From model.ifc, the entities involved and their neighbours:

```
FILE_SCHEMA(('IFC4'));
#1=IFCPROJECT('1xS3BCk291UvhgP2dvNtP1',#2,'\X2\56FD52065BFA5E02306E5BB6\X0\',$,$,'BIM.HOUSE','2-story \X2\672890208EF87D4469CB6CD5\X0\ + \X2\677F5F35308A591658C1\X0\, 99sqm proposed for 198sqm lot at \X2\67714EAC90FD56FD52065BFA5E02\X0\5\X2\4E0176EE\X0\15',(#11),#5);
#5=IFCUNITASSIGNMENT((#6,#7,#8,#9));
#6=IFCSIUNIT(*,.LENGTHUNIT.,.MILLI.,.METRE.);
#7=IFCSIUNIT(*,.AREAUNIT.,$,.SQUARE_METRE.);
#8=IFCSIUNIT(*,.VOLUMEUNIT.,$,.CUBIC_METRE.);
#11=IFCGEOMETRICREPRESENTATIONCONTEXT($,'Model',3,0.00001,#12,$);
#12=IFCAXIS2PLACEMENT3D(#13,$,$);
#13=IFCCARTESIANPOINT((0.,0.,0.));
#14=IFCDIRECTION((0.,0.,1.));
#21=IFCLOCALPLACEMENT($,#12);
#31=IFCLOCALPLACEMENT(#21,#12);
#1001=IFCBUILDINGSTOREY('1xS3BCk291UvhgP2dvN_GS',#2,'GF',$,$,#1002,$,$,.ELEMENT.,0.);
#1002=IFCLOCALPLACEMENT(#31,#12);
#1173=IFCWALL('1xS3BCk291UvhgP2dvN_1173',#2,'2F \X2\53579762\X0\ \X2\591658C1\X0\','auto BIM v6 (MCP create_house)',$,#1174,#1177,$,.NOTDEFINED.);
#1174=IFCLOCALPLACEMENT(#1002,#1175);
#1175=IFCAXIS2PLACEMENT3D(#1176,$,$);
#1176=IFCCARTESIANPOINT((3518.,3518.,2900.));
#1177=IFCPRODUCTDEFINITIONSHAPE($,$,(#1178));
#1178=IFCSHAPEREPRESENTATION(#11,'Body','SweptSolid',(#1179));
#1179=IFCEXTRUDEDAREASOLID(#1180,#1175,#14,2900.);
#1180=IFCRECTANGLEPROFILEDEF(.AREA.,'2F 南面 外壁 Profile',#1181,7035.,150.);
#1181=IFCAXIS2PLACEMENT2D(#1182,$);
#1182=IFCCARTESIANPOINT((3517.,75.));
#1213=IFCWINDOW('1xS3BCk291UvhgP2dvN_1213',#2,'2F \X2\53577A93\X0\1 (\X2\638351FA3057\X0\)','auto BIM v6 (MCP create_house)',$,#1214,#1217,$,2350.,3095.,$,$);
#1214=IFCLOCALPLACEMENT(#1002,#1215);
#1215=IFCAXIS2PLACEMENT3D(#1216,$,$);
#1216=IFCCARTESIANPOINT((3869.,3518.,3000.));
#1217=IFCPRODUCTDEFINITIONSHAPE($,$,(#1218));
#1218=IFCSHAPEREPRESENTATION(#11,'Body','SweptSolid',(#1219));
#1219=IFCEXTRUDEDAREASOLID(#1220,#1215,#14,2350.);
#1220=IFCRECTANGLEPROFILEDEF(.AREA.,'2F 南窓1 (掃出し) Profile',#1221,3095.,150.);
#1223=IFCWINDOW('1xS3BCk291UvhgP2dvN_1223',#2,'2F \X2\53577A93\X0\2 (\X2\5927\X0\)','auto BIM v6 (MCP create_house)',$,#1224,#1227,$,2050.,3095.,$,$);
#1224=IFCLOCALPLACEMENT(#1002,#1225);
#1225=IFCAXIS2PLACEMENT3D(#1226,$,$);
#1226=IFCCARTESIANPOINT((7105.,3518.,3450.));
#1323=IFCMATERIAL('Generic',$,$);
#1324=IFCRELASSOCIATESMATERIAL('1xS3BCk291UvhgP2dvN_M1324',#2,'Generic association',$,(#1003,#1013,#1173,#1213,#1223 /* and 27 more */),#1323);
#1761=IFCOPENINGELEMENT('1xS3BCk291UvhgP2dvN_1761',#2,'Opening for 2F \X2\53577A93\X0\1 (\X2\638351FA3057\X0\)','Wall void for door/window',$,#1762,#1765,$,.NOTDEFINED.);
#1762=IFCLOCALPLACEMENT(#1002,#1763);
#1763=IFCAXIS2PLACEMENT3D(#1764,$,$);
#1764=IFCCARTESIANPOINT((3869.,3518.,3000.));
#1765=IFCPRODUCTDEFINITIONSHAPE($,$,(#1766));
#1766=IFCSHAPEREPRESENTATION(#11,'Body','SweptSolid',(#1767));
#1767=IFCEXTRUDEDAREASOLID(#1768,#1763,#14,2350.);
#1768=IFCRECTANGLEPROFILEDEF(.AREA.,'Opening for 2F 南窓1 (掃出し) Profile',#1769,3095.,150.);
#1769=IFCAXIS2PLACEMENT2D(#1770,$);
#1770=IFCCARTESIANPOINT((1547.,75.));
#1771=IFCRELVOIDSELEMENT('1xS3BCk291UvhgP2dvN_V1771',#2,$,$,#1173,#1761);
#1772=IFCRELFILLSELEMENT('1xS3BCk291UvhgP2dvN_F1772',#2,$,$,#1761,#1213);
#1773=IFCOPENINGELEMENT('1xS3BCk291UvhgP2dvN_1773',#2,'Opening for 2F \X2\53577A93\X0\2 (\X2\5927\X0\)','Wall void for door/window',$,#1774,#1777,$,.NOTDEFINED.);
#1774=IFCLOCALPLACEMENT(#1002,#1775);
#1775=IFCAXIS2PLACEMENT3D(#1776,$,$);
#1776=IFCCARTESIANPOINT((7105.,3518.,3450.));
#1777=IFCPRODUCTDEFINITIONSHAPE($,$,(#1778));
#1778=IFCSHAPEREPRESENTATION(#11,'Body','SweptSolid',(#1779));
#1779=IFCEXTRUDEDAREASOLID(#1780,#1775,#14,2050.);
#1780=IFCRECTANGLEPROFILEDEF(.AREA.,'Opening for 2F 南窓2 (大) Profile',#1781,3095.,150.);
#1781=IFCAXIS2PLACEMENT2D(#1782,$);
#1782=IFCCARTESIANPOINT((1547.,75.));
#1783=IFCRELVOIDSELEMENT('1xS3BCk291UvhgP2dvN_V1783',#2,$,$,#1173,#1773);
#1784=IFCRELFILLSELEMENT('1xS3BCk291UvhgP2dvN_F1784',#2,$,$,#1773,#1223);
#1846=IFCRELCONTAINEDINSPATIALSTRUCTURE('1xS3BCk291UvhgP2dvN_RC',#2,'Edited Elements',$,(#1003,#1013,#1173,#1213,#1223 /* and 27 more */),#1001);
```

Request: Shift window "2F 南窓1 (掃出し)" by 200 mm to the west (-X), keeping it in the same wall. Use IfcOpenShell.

```python
import ifcopenshell
import ifcopenshell.api.geometry
import ifcopenshell.util.placement
import ifcopenshell.util.unit

model = ifcopenshell.open("model.ifc")
unit_scale = ifcopenshell.util.unit.calculate_unit_scale(model)

window = model.by_id(1213)
opening = window.FillsVoids[0].RelatingOpeningElement
wall = opening.VoidsElements[0].RelatingBuildingElement

wall_matrix = ifcopenshell.util.placement.get_local_placement(wall.ObjectPlacement)
shift = wall_matrix[:3, 0] * -0.2 / unit_scale
before = ifcopenshell.util.placement.get_local_placement(window.ObjectPlacement)[:3, 3].copy()

# The window is not placed relative to its opening, so move both.
for product in (opening, window):
    matrix = ifcopenshell.util.placement.get_local_placement(product.ObjectPlacement)
    matrix[:3, 3] += shift
    ifcopenshell.api.geometry.edit_object_placement(model, product=product, matrix=matrix, is_si=False)

after = ifcopenshell.util.placement.get_local_placement(window.ObjectPlacement)[:3, 3]
print("window moved by", (after - before).round(3) + 0.0)

model.write("model_v2.ifc")
```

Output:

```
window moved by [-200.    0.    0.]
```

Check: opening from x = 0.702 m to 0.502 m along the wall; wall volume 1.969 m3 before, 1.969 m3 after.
